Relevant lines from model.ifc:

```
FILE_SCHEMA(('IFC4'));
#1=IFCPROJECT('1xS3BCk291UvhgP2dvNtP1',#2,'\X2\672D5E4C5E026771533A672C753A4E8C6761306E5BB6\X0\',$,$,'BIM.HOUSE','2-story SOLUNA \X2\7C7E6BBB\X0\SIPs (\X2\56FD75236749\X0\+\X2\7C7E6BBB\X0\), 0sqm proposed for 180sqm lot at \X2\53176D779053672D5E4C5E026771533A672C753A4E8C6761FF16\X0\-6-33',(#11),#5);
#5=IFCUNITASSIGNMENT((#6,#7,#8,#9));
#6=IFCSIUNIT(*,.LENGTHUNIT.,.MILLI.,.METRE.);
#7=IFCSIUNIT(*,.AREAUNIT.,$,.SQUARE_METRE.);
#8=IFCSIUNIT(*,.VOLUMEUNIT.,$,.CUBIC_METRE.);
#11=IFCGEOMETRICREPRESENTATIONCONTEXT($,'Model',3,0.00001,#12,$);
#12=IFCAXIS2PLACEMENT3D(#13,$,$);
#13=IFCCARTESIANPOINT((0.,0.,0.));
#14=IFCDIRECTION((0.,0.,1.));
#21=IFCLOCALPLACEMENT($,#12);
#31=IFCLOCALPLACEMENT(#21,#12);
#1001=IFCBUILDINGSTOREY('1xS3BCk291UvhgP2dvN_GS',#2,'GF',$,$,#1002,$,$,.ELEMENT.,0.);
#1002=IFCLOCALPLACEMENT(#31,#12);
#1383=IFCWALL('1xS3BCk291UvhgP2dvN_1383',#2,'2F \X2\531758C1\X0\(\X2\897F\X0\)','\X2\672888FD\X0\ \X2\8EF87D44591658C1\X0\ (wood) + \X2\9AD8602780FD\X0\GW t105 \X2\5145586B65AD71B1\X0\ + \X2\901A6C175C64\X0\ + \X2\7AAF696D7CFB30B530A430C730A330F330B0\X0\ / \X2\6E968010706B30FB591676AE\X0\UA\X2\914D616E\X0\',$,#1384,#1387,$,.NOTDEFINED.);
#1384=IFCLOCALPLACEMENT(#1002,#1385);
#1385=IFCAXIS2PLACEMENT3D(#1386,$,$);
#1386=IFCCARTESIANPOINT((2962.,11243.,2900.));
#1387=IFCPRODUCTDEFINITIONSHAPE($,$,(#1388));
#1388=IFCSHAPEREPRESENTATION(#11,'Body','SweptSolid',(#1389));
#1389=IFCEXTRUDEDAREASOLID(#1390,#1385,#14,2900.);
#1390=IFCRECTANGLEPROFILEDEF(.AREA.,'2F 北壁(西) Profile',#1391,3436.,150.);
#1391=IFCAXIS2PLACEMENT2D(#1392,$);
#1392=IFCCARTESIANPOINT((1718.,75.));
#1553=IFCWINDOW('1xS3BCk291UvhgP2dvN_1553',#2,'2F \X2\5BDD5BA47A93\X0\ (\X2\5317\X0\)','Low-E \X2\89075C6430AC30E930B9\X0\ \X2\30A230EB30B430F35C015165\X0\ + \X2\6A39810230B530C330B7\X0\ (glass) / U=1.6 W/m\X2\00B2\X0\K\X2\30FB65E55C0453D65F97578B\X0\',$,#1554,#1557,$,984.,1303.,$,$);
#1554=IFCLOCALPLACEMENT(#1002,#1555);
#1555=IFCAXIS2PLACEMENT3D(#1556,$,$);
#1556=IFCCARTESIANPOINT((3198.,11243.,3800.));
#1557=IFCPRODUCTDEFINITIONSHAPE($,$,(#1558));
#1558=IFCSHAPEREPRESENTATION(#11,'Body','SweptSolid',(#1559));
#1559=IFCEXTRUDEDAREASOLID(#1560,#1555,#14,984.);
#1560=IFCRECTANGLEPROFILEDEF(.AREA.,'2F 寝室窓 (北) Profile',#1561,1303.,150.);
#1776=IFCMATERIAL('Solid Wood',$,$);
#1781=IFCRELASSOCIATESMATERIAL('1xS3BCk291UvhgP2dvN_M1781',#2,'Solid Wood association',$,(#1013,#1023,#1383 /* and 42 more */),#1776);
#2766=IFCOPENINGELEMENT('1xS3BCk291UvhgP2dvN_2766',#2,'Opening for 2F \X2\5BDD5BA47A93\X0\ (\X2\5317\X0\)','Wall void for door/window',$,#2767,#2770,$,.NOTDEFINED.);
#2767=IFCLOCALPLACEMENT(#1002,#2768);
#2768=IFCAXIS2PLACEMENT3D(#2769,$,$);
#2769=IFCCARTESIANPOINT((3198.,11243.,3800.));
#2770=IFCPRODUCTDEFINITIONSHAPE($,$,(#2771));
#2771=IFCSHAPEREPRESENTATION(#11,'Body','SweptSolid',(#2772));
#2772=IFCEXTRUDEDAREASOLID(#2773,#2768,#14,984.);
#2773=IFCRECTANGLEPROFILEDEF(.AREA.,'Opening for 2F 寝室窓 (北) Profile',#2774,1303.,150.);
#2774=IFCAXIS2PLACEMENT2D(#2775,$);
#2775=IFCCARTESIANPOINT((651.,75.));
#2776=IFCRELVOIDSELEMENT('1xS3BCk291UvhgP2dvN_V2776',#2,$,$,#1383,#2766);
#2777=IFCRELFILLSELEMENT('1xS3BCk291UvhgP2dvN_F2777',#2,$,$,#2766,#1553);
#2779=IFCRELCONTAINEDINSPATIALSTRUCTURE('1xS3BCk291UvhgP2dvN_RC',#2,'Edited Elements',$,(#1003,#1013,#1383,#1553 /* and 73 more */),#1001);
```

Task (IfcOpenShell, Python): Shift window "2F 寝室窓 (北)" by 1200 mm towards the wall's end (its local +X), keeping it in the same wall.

```python
import ifcopenshell
import ifcopenshell.api.geometry
import ifcopenshell.util.placement

model = ifcopenshell.open("model.ifc")

window = model.by_guid("1xS3BCk291UvhgP2dvN_1553")
opening = window.FillsVoids[0].RelatingOpeningElement
wall = opening.VoidsElements[0].RelatingBuildingElement

wall_matrix = ifcopenshell.util.placement.get_local_placement(wall.ObjectPlacement)
shift = wall_matrix[:3, 0] * 1200.0
before = ifcopenshell.util.placement.get_local_placement(window.ObjectPlacement)[:3, 3].copy()

# The window is not placed relative to its opening, so move both.
for product in (opening, window):
    matrix = ifcopenshell.util.placement.get_local_placement(product.ObjectPlacement)
    matrix[:3, 3] += shift
    ifcopenshell.api.geometry.edit_object_placement(model, product=product, matrix=matrix, is_si=False)

after = ifcopenshell.util.placement.get_local_placement(window.ObjectPlacement)[:3, 3]
print("window moved by", (after - before).round(3) + 0.0)

model.write("model_v2.ifc")
```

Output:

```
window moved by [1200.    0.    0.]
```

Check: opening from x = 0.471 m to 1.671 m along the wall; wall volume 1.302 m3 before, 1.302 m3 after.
